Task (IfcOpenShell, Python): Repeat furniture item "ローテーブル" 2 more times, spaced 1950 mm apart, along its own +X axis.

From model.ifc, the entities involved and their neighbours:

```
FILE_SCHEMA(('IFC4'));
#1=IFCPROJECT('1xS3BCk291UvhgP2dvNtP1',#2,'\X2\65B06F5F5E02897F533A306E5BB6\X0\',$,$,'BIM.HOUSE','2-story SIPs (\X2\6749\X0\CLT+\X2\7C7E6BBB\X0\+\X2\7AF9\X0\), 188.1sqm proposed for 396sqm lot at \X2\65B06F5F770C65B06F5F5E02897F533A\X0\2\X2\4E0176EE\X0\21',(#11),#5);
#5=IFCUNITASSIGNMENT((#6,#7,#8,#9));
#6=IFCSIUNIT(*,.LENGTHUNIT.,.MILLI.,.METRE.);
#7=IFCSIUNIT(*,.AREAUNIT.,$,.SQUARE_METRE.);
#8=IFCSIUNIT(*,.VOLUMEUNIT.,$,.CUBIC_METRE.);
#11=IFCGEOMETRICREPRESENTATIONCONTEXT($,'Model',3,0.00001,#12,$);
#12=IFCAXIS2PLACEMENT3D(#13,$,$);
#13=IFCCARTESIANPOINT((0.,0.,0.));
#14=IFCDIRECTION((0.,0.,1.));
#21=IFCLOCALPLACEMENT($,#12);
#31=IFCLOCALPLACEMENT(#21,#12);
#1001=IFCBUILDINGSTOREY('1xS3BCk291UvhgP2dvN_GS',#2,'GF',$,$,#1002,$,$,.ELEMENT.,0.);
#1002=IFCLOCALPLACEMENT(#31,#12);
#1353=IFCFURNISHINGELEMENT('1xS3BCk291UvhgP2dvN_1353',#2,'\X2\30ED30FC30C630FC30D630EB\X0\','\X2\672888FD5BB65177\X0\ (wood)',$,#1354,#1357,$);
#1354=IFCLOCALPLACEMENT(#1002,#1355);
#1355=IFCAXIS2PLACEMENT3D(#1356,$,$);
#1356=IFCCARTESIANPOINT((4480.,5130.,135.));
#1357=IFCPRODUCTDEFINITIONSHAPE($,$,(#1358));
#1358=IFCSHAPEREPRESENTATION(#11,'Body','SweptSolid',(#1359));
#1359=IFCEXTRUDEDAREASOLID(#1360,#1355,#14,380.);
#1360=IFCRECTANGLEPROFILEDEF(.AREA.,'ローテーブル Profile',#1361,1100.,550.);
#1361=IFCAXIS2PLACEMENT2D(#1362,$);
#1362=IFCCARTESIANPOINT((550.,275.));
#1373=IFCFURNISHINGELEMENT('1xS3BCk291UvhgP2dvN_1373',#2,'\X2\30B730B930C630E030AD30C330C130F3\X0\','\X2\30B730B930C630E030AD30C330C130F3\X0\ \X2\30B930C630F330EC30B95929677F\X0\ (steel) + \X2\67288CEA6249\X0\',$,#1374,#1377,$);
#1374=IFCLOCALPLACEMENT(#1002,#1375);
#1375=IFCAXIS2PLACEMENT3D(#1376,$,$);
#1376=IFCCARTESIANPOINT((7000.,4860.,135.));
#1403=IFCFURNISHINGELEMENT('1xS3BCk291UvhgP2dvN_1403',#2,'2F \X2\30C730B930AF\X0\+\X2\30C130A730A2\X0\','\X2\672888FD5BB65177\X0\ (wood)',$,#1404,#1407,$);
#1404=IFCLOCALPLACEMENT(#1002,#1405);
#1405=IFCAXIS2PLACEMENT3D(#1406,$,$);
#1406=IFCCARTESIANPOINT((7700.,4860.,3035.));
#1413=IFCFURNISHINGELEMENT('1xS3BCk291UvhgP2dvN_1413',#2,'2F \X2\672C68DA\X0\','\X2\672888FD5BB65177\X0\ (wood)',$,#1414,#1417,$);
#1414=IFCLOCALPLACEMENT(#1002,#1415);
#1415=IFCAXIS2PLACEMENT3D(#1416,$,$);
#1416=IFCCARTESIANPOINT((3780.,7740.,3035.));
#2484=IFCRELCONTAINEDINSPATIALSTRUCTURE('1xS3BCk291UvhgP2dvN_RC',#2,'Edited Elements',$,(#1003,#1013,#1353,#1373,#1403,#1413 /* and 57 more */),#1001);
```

```python
import ifcopenshell
import ifcopenshell.api.geometry
import ifcopenshell.api.root
import ifcopenshell.util.element
import ifcopenshell.util.placement

model = ifcopenshell.open("model.ifc")


def reuse_history(source, copy):
    """copy_class also copies each property set's owner history, people and application; keep the originals."""
    for rel in copy.IsDefinedBy:
        if rel.is_a("IfcRelDefinesByProperties") and (history := rel.RelatingPropertyDefinition.OwnerHistory):
            rel.RelatingPropertyDefinition.OwnerHistory = source.OwnerHistory
            ifcopenshell.util.element.remove_deep2(model, history)


source = model.by_guid("1xS3BCk291UvhgP2dvN_1353")
base = ifcopenshell.util.placement.get_local_placement(source.ObjectPlacement)
step = base[:3, 0] * 1950.0

for i in range(1, 3):
    copy = ifcopenshell.api.root.copy_class(model, product=source)
    copy.Representation = ifcopenshell.util.element.copy_deep(
        model, source.Representation, exclude=["IfcGeometricRepresentationContext", "IfcRepresentationMap"]
    )
    reuse_history(source, copy)
    matrix = base.copy()
    matrix[:3, 3] += i * step
    print("added at", matrix[:3, 3].round(3) + 0.0)
    ifcopenshell.api.geometry.edit_object_placement(model, product=copy, matrix=matrix, is_si=False)

model.write("model_rev.ifc")
```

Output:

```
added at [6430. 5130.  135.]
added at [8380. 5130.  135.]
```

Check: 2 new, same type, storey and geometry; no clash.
